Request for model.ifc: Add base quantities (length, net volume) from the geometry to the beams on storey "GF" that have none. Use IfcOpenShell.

First a look at what the model holds.

```python
import ifcopenshell
import ifcopenshell.util.element
import ifcopenshell.util.unit

model = ifcopenshell.open("model.ifc")
print(model.schema)
for unit_type in ("LENGTHUNIT", "AREAUNIT", "VOLUMEUNIT"):
    print(unit_type, ifcopenshell.util.unit.calculate_unit_scale(model, unit_type))
storey = next(s for s in model.by_type("IfcBuildingStorey") if s.Name == "GF")
beams = [e for e in ifcopenshell.util.element.get_decomposition(storey) if e.is_a("IfcBeam")]
for e in sorted(beams, key=lambda e: e.id()):
    print(e.id(), e.is_a(), e.Name, list(ifcopenshell.util.element.get_psets(e, qtos_only=True)), sep=" | ")
```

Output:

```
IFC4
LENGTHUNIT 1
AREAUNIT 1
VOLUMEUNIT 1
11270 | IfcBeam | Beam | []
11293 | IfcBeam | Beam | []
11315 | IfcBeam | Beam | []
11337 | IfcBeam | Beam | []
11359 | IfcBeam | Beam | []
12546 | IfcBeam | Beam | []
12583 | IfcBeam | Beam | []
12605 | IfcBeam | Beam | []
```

```python
import ifcopenshell
import ifcopenshell.api.pset
import ifcopenshell.geom
import ifcopenshell.util.element
import ifcopenshell.util.shape
import ifcopenshell.util.unit

model = ifcopenshell.open("model.ifc")
unit_scale = ifcopenshell.util.unit.calculate_unit_scale(model)
volume_scale = ifcopenshell.util.unit.calculate_unit_scale(model, "VOLUMEUNIT")
settings = ifcopenshell.geom.settings()

storey = next(s for s in model.by_type("IfcBuildingStorey") if s.Name == "GF")
beams = [e for e in ifcopenshell.util.element.get_decomposition(storey) if e.is_a("IfcBeam")]

for e in sorted(beams, key=lambda e: e.id()):
    if ifcopenshell.util.element.get_psets(e, qtos_only=True, should_inherit=False):
        continue
    # Geometry comes back in metres, in the element's own axes.
    shape = ifcopenshell.geom.create_shape(settings, e)
    values = {
        "Length": ifcopenshell.util.shape.get_max_xyz(shape.geometry) / unit_scale,
        "NetVolume": ifcopenshell.util.shape.get_volume(shape.geometry) / volume_scale,
    }
    qto = ifcopenshell.api.pset.add_qto(model, product=e, name="Qto_BeamBaseQuantities")
    ifcopenshell.api.pset.edit_qto(model, qto=qto, properties=values)
    print(e.id(), {k: round(v, 3) for k, v in values.items()})

model.write("model_rev.ifc")
```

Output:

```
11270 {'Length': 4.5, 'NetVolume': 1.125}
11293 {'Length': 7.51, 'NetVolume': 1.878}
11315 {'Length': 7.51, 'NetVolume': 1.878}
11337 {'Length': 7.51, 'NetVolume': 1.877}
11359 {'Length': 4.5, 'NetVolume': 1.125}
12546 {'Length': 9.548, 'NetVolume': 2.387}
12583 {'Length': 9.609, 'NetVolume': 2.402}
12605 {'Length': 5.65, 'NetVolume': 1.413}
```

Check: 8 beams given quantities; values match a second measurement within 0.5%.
